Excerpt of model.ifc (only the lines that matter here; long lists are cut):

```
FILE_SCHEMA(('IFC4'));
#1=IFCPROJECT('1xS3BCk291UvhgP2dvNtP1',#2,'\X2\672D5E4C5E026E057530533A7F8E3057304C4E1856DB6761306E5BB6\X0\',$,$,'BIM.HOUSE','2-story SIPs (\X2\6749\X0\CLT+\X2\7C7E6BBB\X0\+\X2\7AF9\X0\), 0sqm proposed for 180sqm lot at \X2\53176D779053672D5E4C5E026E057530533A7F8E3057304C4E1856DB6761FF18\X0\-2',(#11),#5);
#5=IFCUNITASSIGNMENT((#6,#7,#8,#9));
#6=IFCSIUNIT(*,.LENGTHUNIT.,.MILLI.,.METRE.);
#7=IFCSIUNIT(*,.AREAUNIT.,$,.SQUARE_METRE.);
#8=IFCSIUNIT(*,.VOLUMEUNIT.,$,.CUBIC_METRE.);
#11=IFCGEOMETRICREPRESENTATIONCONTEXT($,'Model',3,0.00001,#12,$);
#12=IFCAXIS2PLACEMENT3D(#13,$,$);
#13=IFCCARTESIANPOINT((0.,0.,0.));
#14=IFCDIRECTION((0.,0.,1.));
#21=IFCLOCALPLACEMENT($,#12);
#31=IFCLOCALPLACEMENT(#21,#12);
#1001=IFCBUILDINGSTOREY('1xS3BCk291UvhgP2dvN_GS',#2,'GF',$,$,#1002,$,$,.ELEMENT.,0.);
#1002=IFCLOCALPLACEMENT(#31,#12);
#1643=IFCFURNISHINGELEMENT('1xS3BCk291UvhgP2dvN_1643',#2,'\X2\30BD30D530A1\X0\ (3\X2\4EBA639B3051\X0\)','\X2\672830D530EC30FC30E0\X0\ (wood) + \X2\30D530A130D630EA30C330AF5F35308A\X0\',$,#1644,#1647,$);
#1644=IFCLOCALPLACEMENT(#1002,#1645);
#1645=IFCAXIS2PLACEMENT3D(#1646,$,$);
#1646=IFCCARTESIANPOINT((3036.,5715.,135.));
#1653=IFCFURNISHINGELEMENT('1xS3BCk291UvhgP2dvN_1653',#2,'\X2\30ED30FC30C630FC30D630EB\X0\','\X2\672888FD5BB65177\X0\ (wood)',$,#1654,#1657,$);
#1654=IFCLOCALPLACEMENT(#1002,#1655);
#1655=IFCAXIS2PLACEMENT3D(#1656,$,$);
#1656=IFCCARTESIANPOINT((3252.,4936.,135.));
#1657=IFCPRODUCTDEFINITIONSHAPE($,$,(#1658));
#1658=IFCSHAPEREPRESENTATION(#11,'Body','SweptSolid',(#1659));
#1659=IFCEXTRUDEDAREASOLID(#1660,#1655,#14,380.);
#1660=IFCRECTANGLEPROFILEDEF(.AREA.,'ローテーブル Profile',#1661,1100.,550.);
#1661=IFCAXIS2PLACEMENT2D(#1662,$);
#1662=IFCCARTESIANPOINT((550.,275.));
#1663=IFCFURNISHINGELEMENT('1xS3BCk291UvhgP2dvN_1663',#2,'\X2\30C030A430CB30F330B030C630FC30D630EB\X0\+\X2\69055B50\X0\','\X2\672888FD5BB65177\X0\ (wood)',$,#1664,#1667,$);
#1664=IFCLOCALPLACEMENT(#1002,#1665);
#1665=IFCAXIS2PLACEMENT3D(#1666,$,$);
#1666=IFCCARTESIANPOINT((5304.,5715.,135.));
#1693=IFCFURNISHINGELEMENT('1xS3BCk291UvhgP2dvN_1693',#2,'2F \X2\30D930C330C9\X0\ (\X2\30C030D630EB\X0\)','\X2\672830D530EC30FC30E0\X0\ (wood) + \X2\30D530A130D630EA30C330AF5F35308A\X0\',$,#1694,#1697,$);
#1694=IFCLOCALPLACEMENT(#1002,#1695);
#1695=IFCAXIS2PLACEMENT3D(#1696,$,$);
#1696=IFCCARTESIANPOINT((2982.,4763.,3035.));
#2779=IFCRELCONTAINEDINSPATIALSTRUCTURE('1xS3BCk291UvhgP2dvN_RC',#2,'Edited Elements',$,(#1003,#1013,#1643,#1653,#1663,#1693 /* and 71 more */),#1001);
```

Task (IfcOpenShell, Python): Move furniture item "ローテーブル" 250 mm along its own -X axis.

```python
import ifcopenshell
import ifcopenshell.api.geometry
import ifcopenshell.util.placement
import ifcopenshell.util.unit

model = ifcopenshell.open("model.ifc")
unit_scale = ifcopenshell.util.unit.calculate_unit_scale(model)

item = model.by_guid("1xS3BCk291UvhgP2dvN_1653")
matrix = ifcopenshell.util.placement.get_local_placement(item.ObjectPlacement)
matrix[:3, 3] -= matrix[:3, 0] * 0.25 / unit_scale
ifcopenshell.api.geometry.edit_object_placement(model, product=item, matrix=matrix, is_si=False)

print(ifcopenshell.util.placement.get_local_placement(item.ObjectPlacement).round(3) + 0.0)

model.write("model_v2.ifc")
```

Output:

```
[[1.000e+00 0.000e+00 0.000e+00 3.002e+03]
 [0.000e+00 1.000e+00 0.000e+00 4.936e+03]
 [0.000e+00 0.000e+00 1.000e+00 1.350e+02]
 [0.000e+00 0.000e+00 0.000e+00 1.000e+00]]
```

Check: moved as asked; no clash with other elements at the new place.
